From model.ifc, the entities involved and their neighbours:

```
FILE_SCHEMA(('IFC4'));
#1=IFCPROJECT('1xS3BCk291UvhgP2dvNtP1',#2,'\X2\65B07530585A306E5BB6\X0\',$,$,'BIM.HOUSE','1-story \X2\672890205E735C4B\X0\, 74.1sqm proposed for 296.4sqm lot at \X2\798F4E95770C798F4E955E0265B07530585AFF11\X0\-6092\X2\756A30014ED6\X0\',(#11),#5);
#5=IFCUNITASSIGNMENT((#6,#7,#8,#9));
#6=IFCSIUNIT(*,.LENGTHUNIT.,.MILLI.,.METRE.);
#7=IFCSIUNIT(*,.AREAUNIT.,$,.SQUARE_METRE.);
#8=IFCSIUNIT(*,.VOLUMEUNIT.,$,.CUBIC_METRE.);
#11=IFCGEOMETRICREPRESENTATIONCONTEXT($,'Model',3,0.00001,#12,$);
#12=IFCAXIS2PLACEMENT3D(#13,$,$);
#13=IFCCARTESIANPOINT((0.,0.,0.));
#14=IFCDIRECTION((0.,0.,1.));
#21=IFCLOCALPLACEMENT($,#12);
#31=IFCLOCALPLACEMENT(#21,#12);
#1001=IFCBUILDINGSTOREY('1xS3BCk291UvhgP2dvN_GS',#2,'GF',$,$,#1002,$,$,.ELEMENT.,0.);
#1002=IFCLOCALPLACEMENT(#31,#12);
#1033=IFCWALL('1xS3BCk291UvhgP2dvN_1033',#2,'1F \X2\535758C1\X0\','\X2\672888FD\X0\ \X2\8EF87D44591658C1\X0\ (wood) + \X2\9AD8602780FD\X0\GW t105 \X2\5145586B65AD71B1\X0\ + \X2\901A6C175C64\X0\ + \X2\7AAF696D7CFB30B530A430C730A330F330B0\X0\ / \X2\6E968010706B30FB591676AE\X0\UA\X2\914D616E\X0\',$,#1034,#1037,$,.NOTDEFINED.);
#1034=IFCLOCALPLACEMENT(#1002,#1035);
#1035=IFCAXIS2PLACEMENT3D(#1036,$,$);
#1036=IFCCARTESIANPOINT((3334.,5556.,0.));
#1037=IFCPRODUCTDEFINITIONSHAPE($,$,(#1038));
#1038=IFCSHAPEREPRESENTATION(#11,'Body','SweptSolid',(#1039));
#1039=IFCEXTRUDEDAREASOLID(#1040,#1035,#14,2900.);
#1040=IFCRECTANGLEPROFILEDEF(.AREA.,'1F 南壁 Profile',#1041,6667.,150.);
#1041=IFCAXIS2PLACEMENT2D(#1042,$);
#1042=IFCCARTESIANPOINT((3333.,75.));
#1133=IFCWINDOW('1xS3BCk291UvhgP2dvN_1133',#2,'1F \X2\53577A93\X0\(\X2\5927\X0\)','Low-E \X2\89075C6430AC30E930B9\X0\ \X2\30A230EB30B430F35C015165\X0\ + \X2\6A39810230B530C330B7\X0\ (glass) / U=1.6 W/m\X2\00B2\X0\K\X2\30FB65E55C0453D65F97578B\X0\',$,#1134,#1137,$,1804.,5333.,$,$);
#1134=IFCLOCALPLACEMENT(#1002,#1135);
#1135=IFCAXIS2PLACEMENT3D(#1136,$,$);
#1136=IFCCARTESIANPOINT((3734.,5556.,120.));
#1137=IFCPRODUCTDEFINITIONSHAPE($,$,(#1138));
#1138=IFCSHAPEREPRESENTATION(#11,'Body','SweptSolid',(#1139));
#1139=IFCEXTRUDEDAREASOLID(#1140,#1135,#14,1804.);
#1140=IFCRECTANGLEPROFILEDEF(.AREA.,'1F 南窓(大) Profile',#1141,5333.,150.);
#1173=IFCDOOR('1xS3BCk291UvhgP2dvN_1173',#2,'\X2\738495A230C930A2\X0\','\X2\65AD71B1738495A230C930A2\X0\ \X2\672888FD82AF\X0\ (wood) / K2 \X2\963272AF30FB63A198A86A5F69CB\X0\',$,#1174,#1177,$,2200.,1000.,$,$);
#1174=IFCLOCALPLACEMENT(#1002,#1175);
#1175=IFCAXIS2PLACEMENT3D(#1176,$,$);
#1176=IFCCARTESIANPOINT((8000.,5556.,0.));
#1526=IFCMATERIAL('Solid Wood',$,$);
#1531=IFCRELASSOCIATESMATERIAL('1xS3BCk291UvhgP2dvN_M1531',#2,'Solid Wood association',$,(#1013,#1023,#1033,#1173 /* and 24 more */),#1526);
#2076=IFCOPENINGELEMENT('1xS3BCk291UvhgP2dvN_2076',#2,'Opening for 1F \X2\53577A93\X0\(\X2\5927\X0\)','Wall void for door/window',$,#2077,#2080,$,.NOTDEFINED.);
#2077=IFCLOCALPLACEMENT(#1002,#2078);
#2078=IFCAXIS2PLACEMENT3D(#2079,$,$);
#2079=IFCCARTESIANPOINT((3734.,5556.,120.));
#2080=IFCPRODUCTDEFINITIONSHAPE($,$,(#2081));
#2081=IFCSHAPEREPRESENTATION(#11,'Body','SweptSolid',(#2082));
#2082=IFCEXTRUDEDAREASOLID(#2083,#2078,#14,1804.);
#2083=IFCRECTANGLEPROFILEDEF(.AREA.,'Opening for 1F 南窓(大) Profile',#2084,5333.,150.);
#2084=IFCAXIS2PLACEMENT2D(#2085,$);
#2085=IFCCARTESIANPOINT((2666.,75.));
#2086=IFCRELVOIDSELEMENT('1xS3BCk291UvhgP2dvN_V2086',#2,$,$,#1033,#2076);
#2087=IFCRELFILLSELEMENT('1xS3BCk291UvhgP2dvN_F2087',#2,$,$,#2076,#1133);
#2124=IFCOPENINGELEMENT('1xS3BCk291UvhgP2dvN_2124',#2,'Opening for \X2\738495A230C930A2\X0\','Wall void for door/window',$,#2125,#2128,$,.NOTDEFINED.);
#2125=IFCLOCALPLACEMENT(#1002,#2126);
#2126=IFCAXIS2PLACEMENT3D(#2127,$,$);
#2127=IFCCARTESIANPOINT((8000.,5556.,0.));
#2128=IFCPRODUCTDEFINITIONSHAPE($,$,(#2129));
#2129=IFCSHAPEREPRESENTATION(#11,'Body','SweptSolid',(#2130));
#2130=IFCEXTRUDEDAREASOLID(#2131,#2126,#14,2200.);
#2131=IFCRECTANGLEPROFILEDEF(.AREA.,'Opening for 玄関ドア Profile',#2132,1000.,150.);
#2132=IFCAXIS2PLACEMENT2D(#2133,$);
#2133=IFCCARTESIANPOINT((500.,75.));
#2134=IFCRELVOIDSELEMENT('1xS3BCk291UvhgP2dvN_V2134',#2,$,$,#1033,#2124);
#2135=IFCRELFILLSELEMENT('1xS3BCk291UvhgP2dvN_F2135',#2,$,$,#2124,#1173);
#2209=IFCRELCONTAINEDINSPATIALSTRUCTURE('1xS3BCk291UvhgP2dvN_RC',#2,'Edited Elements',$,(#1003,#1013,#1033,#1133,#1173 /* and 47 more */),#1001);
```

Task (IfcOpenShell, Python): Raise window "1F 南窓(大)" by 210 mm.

```python
import numpy as np
import ifcopenshell
import ifcopenshell.api.geometry
import ifcopenshell.util.placement
import ifcopenshell.util.unit

model = ifcopenshell.open("model.ifc")
unit_scale = ifcopenshell.util.unit.calculate_unit_scale(model)

window = model.by_id(1133)
opening = window.FillsVoids[0].RelatingOpeningElement
dz = 210.0

shift = np.array([0.0, 0.0, dz])
# The window is not placed relative to its opening, so move both.
for product in (opening, window):
    matrix = ifcopenshell.util.placement.get_local_placement(product.ObjectPlacement)
    matrix[:3, 3] += shift
    ifcopenshell.api.geometry.edit_object_placement(model, product=product, matrix=matrix, is_si=False)

print(f"moved by {dz * unit_scale:+.3f} m")

model.write("model-out.ifc")
```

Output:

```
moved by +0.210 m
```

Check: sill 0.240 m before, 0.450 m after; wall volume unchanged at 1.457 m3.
